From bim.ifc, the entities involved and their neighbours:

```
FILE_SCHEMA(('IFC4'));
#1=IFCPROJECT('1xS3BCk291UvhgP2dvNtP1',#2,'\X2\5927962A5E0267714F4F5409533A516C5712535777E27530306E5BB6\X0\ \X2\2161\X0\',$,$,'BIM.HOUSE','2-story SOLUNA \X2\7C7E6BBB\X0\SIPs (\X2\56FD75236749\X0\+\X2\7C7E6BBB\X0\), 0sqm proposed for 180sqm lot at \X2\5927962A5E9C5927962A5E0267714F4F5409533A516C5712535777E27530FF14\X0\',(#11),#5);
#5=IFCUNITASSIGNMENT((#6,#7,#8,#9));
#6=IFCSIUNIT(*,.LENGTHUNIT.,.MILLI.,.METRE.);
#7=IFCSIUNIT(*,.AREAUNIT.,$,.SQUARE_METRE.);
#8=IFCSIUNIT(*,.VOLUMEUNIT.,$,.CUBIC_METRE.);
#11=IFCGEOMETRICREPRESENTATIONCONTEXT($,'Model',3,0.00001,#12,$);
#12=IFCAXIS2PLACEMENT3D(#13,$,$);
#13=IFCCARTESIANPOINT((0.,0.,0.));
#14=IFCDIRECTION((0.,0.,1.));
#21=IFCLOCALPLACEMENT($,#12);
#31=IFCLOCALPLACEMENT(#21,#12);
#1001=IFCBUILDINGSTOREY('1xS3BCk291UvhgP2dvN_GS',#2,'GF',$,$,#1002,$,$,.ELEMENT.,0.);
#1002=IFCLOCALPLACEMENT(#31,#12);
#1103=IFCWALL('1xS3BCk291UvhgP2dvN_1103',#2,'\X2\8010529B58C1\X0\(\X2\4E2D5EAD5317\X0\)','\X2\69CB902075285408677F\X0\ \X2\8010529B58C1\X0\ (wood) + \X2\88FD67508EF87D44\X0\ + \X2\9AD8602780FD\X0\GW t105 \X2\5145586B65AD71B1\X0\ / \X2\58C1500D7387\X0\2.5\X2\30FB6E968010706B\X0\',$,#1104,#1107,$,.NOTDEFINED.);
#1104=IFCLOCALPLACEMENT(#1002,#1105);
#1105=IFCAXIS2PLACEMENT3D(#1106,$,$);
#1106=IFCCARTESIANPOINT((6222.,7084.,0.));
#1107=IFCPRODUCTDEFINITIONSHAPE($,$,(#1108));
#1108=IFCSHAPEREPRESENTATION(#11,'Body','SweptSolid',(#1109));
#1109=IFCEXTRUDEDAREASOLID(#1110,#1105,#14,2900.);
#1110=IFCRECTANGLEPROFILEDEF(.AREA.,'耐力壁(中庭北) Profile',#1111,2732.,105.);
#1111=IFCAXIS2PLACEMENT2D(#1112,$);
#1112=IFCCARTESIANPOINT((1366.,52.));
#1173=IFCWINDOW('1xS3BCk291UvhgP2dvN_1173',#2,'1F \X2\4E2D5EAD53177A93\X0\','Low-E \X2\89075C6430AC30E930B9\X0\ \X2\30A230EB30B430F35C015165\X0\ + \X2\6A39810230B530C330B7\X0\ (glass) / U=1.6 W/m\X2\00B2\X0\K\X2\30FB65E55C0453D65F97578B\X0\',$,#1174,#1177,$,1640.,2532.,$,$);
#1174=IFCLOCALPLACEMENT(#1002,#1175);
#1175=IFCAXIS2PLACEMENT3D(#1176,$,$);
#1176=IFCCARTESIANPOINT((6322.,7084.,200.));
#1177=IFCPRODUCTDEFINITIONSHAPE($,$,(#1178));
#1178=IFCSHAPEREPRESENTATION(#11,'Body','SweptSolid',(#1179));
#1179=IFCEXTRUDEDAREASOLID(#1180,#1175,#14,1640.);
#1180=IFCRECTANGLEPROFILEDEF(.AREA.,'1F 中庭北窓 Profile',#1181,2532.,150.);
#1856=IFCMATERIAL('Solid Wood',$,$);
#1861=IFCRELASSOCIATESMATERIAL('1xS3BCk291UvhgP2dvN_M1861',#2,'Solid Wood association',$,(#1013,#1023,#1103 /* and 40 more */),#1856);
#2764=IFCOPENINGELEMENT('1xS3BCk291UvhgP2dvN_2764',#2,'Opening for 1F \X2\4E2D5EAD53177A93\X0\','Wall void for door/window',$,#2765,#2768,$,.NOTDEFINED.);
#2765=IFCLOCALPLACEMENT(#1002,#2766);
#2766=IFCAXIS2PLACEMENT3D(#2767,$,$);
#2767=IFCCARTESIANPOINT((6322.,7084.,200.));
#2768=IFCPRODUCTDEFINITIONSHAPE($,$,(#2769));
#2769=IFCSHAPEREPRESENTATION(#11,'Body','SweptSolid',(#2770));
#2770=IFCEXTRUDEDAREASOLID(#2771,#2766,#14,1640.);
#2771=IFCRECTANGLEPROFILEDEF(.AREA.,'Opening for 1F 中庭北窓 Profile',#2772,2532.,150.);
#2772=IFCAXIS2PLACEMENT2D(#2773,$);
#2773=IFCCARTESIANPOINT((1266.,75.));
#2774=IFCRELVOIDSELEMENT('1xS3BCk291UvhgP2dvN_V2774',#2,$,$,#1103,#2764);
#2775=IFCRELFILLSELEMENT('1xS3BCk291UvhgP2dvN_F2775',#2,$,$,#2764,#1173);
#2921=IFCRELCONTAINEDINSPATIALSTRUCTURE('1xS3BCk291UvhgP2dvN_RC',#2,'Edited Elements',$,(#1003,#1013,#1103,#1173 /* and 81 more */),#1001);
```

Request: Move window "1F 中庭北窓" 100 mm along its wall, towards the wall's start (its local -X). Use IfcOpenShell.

```python
import ifcopenshell
import ifcopenshell.api.geometry
import ifcopenshell.util.placement
import ifcopenshell.util.unit

model = ifcopenshell.open("bim.ifc")
unit_scale = ifcopenshell.util.unit.calculate_unit_scale(model)

window = model.by_guid("1xS3BCk291UvhgP2dvN_1173")
opening = window.FillsVoids[0].RelatingOpeningElement
wall = opening.VoidsElements[0].RelatingBuildingElement

wall_matrix = ifcopenshell.util.placement.get_local_placement(wall.ObjectPlacement)
shift = wall_matrix[:3, 0] * -0.1 / unit_scale
before = ifcopenshell.util.placement.get_local_placement(window.ObjectPlacement)[:3, 3].copy()

# The window is not placed relative to its opening, so move both.
for product in (opening, window):
    matrix = ifcopenshell.util.placement.get_local_placement(product.ObjectPlacement)
    matrix[:3, 3] += shift
    ifcopenshell.api.geometry.edit_object_placement(model, product=product, matrix=matrix, is_si=False)

after = ifcopenshell.util.placement.get_local_placement(window.ObjectPlacement)[:3, 3]
print("window moved by", (after - before).round(3) + 0.0)

model.write("bim_rev.ifc")
```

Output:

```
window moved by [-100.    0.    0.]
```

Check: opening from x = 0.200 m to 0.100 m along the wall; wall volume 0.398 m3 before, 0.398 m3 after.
